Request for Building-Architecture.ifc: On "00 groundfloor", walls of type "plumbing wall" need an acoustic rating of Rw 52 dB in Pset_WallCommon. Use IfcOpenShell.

First a look at what the model holds.

```python
import ifcopenshell
import ifcopenshell.util.element

model = ifcopenshell.open("Building-Architecture.ifc")
print(model.schema)
storey = next(s for s in model.by_type("IfcBuildingStorey") if s.Name == "00 groundfloor")
walls = [e for e in ifcopenshell.util.element.get_decomposition(storey) if e.is_a("IfcWall")]
seen = {}
for e in walls:
    element_type = ifcopenshell.util.element.get_type(e)
    key = (element_type.Name if element_type != e and element_type else None, ifcopenshell.util.element.get_pset(e, "Pset_WallCommon", "AcousticRating"))
    seen[key] = seen.get(key, 0) + 1
for (name, value), count in sorted(seen.items(), key=str):
    print(count, "x", name, "|", value)
```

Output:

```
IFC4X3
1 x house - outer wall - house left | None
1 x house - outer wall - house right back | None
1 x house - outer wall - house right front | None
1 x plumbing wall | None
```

```python
import ifcopenshell
import ifcopenshell.api.pset
import ifcopenshell.util.element

model = ifcopenshell.open("Building-Architecture.ifc")

storey = next(s for s in model.by_type("IfcBuildingStorey") if s.Name == "00 groundfloor")
walls = [e for e in ifcopenshell.util.element.get_decomposition(storey) if e.is_a("IfcWall")]

count = 0
for e in walls:
    element_type = ifcopenshell.util.element.get_type(e)
    if element_type in (None, e) or element_type.Name != "plumbing wall":
        continue
    # add_pset returns the element's existing set when there is one.
    pset = ifcopenshell.api.pset.add_pset(model, product=e, name="Pset_WallCommon")
    ifcopenshell.api.pset.edit_pset(model, pset=pset, properties={"AcousticRating": "Rw 52 dB"})
    count += 1

print(count, "walls updated")

model.write("Building-Architecture_updated.ifc")
```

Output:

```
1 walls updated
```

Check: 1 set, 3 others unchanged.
